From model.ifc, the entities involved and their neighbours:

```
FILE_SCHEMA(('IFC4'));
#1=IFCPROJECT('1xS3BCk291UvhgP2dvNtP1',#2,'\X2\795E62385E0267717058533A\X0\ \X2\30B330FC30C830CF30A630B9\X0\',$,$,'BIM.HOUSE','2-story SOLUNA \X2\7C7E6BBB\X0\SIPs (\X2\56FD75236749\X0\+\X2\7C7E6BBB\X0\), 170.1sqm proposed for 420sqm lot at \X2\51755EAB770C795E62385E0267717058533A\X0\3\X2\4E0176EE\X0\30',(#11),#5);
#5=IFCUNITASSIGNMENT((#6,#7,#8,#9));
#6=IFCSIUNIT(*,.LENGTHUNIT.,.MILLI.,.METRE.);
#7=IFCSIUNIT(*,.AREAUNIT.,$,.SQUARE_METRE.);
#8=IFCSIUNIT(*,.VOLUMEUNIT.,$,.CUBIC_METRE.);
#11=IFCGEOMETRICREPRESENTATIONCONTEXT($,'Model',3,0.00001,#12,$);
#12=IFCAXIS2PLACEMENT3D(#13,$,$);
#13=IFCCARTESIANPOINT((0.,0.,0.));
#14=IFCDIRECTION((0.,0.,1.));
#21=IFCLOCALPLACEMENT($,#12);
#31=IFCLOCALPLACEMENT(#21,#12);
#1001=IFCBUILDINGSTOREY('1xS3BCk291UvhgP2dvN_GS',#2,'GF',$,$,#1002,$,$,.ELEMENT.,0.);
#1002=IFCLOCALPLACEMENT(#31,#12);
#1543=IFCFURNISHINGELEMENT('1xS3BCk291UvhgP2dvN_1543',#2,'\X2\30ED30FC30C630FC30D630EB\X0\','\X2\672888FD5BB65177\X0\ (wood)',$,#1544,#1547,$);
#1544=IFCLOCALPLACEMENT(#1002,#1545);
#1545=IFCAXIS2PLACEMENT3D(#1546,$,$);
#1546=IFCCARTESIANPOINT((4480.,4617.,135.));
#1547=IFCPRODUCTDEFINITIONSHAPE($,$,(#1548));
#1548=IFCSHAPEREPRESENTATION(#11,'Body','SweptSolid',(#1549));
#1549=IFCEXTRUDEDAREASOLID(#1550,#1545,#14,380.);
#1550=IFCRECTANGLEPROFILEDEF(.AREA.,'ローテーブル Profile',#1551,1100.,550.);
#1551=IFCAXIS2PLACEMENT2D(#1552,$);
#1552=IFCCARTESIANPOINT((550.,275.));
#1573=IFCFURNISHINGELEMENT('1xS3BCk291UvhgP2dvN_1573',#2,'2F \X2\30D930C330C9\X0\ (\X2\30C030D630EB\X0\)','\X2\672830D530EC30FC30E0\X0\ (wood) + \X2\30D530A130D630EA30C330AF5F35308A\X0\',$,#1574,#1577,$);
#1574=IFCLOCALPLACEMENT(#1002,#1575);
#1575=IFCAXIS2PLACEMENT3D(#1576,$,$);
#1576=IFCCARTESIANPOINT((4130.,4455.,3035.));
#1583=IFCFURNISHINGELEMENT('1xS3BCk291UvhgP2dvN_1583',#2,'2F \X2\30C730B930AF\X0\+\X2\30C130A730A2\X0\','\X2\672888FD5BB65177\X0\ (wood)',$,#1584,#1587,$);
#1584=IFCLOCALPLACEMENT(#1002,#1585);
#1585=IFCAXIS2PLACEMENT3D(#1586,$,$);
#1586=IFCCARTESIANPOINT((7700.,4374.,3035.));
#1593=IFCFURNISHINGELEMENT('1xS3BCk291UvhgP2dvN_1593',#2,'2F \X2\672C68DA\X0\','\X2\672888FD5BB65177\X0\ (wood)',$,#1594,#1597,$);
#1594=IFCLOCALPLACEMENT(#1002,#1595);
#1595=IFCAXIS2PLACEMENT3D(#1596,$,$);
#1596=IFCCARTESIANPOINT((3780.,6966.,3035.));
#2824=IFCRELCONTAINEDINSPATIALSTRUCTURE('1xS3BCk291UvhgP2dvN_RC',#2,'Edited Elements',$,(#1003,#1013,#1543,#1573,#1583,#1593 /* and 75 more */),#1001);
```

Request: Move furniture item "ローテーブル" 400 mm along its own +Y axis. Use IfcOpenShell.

```python
import ifcopenshell
import ifcopenshell.api.geometry
import ifcopenshell.util.placement
import ifcopenshell.util.unit

model = ifcopenshell.open("model.ifc")
unit_scale = ifcopenshell.util.unit.calculate_unit_scale(model)

item = model.by_guid("1xS3BCk291UvhgP2dvN_1543")
matrix = ifcopenshell.util.placement.get_local_placement(item.ObjectPlacement)
matrix[:3, 3] += matrix[:3, 1] * 0.4 / unit_scale
ifcopenshell.api.geometry.edit_object_placement(model, product=item, matrix=matrix, is_si=False)

print(ifcopenshell.util.placement.get_local_placement(item.ObjectPlacement).round(3) + 0.0)

model.write("model-out.ifc")
```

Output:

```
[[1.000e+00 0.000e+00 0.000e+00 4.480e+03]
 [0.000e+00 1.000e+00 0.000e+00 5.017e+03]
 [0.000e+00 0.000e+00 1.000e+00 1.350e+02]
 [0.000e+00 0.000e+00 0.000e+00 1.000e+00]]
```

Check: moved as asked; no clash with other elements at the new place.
